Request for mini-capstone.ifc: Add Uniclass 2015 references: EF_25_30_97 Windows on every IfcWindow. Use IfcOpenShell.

First a look at what the model holds.

```python
import ifcopenshell

model = ifcopenshell.open("mini-capstone.ifc")
print(model.schema)
print("classifications:", [c.Name for c in model.by_type("IfcClassification")])
for ifc_class in ("IfcDoor", "IfcRoof", "IfcStair", "IfcWall", "IfcWindow"):
    print(ifc_class, len(model.by_type(ifc_class)))
```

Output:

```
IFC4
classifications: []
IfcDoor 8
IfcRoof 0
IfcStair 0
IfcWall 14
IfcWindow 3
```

```python
import ifcopenshell
import ifcopenshell.api.classification

model = ifcopenshell.open("mini-capstone.ifc")

system = ifcopenshell.api.classification.add_classification(model, classification="Uniclass 2015")

codes = {
    "IfcWindow": ("EF_25_30_97", "Windows"),
}
for ifc_class, (code, name) in codes.items():
    products = model.by_type(ifc_class)
    ifcopenshell.api.classification.add_reference(
        model, products=products, classification=system, identification=code, name=name
    )
    print(code, len(products))

model.write("mini-capstone_v2.ifc")
```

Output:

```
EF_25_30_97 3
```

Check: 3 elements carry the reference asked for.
